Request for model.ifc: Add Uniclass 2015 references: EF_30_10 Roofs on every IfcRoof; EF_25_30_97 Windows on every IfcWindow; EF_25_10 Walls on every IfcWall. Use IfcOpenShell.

First a look at what the model holds.

```python
import ifcopenshell

model = ifcopenshell.open("model.ifc")
print(model.schema)
print("classifications:", [c.Name for c in model.by_type("IfcClassification")])
for ifc_class in ("IfcDoor", "IfcRoof", "IfcStair", "IfcWall", "IfcWindow"):
    print(ifc_class, len(model.by_type(ifc_class)))
```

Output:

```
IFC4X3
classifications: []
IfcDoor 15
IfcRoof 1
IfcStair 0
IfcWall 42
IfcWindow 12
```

```python
import ifcopenshell
import ifcopenshell.api.classification

model = ifcopenshell.open("model.ifc")

system = ifcopenshell.api.classification.add_classification(model, classification="Uniclass 2015")

codes = {
    "IfcRoof": ("EF_30_10", "Roofs"),
    "IfcWindow": ("EF_25_30_97", "Windows"),
    "IfcWall": ("EF_25_10", "Walls"),
}
for ifc_class, (code, name) in codes.items():
    products = model.by_type(ifc_class)
    ifcopenshell.api.classification.add_reference(
        model, products=products, classification=system, identification=code, name=name
    )
    print(code, len(products))

model.write("model_v2.ifc")
```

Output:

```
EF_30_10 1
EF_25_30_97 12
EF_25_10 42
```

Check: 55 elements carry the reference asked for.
